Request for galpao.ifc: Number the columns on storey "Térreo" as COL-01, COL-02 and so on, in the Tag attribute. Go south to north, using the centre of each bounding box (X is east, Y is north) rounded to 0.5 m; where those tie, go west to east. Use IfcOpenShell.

First a look at what the model holds.

```python
import ifcopenshell
import ifcopenshell.util.element
import ifcopenshell.util.placement

model = ifcopenshell.open("galpao.ifc")
print(model.schema)
storey = next(s for s in model.by_type("IfcBuildingStorey") if s.Name == "Térreo")
columns = [e for e in ifcopenshell.util.element.get_decomposition(storey) if e.is_a("IfcColumn")]
for e in sorted(columns, key=lambda e: e.id()):
    origin = ifcopenshell.util.placement.get_local_placement(e.ObjectPlacement)[:3, 3]
    print(e.id(), e.Tag, e.Name, origin.round(2) + 0.0, sep=" | ")
```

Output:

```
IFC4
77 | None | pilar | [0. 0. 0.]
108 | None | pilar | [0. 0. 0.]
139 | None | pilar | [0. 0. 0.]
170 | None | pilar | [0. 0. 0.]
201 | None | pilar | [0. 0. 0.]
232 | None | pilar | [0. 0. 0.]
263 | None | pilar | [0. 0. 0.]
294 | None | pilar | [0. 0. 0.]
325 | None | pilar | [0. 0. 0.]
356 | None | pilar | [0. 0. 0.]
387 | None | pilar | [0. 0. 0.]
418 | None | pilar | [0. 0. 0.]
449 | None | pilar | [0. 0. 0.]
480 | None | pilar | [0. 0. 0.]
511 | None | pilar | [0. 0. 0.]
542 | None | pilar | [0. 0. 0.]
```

```python
import ifcopenshell
import ifcopenshell.geom
import ifcopenshell.util.element
import ifcopenshell.util.shape

model = ifcopenshell.open("galpao.ifc")
settings = ifcopenshell.geom.settings()
settings.set("use-world-coords", True)


def centre(element):
    shape = ifcopenshell.geom.create_shape(settings, element)
    return ifcopenshell.util.shape.get_bbox_centroid(shape.geometry)


storey = next(s for s in model.by_type("IfcBuildingStorey") if s.Name == "Térreo")
columns = [e for e in ifcopenshell.util.element.get_decomposition(storey) if e.is_a("IfcColumn")]

# Insertion points can sit at a corner or the storey origin, so sort by the geometry (in metres).
centres = {e: centre(e) for e in columns}
columns.sort(key=lambda e: (round(centres[e][1] / 0.5), centres[e][0]))

for i, e in enumerate(columns, start=1):
    number = f"COL-{i:02d}"
    e.Tag = number
    print(e.id(), number)

model.write("galpao_rev.ifc")
```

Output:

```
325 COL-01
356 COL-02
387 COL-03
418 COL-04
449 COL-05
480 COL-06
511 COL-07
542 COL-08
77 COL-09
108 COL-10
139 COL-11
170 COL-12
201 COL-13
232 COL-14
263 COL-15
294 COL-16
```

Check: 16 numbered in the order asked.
